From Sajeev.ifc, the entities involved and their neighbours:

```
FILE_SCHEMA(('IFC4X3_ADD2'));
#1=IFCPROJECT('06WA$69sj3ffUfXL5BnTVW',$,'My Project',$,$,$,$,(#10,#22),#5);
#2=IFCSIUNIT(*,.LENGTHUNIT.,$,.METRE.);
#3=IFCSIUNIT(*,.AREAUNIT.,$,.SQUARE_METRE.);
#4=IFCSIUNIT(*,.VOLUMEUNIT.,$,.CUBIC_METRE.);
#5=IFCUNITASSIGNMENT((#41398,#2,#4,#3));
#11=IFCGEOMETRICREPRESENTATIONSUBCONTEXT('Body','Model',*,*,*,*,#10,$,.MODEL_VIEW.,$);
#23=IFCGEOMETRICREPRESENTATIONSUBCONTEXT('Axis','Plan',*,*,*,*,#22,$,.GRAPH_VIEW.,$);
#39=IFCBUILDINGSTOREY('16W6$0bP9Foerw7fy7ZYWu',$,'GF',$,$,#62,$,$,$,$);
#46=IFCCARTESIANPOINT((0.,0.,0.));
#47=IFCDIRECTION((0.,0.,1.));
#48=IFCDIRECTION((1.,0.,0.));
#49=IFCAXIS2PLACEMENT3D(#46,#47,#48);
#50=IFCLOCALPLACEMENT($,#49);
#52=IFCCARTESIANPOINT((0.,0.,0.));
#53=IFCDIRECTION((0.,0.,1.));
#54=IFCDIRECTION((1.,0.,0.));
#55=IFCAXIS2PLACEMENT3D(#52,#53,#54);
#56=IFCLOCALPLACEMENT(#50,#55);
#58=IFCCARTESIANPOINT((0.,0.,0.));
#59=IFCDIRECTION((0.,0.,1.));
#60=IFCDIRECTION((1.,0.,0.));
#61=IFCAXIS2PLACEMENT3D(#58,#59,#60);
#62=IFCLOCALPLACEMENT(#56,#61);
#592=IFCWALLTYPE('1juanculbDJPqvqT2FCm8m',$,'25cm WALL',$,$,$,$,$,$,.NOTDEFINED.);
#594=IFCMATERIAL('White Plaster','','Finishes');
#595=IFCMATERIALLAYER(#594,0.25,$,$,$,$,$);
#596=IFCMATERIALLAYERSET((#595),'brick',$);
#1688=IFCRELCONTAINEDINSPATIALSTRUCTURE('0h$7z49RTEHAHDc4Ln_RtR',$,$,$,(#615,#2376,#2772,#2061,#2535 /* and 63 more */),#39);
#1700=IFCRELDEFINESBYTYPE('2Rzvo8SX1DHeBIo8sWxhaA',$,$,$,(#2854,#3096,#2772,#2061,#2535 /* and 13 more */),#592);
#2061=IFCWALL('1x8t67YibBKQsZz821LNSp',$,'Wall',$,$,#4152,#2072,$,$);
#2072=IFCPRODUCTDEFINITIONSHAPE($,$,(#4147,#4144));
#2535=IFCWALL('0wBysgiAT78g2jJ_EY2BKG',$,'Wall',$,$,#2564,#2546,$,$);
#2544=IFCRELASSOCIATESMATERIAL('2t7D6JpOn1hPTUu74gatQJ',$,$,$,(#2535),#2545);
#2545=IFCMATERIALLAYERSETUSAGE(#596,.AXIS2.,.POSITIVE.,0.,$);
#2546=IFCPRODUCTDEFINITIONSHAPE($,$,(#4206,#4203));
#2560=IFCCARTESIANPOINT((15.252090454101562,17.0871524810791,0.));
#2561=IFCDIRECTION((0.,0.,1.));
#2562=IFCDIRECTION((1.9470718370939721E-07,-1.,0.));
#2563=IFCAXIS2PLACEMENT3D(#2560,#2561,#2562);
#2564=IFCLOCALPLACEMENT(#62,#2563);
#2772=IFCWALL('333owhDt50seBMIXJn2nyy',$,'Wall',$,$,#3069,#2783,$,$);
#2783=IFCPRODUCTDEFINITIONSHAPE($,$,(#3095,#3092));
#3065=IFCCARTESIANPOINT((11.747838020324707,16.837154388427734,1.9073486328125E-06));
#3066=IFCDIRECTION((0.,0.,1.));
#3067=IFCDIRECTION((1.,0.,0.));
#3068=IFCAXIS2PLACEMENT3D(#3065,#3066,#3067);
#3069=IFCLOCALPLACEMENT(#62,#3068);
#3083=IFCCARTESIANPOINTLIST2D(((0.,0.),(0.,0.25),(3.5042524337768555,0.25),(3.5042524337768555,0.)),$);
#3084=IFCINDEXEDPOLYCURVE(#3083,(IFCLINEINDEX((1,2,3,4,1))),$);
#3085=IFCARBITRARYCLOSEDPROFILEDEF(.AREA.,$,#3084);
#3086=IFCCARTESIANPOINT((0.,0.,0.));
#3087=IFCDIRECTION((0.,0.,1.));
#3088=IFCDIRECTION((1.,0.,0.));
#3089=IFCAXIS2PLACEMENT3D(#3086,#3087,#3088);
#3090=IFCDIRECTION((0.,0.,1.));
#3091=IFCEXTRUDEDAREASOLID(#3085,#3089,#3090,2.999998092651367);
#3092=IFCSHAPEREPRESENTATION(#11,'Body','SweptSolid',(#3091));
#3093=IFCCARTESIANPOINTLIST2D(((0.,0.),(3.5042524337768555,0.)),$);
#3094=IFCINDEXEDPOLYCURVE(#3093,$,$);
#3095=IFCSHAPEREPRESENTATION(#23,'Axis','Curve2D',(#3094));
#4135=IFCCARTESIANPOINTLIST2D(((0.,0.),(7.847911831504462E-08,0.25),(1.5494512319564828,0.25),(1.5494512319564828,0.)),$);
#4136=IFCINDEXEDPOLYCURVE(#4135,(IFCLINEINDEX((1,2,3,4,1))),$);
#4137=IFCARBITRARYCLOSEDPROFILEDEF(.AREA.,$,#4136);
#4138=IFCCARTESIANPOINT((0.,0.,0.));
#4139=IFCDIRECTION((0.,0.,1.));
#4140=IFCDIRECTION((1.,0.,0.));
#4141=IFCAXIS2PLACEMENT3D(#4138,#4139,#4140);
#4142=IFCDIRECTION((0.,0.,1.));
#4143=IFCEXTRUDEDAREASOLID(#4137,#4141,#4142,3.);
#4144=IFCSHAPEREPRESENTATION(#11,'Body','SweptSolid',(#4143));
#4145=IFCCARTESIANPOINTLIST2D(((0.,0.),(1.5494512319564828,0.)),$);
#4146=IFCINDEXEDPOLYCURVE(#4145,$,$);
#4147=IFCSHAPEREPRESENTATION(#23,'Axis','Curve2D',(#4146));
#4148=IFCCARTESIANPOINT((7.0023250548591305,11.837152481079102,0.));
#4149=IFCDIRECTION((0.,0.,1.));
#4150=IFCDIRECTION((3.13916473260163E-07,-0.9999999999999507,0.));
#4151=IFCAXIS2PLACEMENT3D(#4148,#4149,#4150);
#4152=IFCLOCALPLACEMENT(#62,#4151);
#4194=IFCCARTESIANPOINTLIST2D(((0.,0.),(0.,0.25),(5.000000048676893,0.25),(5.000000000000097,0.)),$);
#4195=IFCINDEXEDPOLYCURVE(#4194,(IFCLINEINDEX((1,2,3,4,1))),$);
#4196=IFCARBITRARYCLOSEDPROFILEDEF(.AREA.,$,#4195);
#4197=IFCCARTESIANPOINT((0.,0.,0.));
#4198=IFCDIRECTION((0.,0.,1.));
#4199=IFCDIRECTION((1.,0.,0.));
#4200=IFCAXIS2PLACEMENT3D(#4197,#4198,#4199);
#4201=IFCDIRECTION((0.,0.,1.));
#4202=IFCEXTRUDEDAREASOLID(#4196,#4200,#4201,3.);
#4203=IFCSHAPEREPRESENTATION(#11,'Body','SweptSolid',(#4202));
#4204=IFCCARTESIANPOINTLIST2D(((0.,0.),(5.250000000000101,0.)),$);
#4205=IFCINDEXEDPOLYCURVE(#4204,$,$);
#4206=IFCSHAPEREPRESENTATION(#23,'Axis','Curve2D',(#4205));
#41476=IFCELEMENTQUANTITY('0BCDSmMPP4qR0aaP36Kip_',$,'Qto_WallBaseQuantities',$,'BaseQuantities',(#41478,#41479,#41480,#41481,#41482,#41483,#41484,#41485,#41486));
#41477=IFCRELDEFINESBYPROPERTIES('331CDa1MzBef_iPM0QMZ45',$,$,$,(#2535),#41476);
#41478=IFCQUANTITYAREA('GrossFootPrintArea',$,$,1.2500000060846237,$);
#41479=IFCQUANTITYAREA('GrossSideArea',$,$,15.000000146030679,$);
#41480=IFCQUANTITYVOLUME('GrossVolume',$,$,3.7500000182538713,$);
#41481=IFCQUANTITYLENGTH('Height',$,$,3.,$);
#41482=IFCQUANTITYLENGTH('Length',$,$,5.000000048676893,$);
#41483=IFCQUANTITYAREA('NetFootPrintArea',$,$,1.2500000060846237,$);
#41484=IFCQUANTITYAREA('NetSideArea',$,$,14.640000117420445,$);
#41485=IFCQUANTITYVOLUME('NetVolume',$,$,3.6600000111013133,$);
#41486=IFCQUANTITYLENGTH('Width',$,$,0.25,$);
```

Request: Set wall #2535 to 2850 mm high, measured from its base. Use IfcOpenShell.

```python
import ifcopenshell
import ifcopenshell.api.pset
import ifcopenshell.geom
import ifcopenshell.util.element
import ifcopenshell.util.representation
import ifcopenshell.util.shape
import ifcopenshell.util.unit

model = ifcopenshell.open("Sajeev.ifc")
unit_scale = ifcopenshell.util.unit.calculate_unit_scale(model)
area_scale = ifcopenshell.util.unit.calculate_unit_scale(model, "AREAUNIT")
volume_scale = ifcopenshell.util.unit.calculate_unit_scale(model, "VOLUMEUNIT")
settings = ifcopenshell.geom.settings()


def volume(element):
    """Net volume in cubic metres, openings subtracted."""
    shape = ifcopenshell.geom.create_shape(settings, element)
    return ifcopenshell.util.shape.get_volume(shape.geometry)


wall = model.by_guid("0wBysgiAT78g2jJ_EY2BKG")
before = volume(wall)

body = ifcopenshell.util.representation.get_representation(wall, "Model", "Body")
solid = body.Items[0]
old_height = solid.Depth
solid.Depth = 2.85 / unit_scale
after = volume(wall)
thickness = 0.25  # wall thickness in metres

# Update the stored height, areas and volumes.
qto = model.by_id(ifcopenshell.util.element.get_pset(wall, "Qto_WallBaseQuantities", should_inherit=False)["id"])
ifcopenshell.api.pset.edit_qto(model, qto=qto, properties={
    "GrossSideArea": ifcopenshell.util.element.get_pset(wall, "Qto_WallBaseQuantities", "GrossSideArea") * solid.Depth / old_height,
    "GrossVolume": ifcopenshell.util.element.get_pset(wall, "Qto_WallBaseQuantities", "GrossVolume") * solid.Depth / old_height,
    "Height": solid.Depth,
    "NetSideArea": after / thickness / area_scale,
    "NetVolume": after / volume_scale,
})

print(f"height {old_height:g} -> {solid.Depth:g}, volume {before:.3f} -> {after:.3f} m3")

model.write("Sajeev_edited.ifc")
```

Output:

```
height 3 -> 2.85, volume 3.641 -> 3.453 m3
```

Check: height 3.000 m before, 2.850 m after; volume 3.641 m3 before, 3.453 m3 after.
